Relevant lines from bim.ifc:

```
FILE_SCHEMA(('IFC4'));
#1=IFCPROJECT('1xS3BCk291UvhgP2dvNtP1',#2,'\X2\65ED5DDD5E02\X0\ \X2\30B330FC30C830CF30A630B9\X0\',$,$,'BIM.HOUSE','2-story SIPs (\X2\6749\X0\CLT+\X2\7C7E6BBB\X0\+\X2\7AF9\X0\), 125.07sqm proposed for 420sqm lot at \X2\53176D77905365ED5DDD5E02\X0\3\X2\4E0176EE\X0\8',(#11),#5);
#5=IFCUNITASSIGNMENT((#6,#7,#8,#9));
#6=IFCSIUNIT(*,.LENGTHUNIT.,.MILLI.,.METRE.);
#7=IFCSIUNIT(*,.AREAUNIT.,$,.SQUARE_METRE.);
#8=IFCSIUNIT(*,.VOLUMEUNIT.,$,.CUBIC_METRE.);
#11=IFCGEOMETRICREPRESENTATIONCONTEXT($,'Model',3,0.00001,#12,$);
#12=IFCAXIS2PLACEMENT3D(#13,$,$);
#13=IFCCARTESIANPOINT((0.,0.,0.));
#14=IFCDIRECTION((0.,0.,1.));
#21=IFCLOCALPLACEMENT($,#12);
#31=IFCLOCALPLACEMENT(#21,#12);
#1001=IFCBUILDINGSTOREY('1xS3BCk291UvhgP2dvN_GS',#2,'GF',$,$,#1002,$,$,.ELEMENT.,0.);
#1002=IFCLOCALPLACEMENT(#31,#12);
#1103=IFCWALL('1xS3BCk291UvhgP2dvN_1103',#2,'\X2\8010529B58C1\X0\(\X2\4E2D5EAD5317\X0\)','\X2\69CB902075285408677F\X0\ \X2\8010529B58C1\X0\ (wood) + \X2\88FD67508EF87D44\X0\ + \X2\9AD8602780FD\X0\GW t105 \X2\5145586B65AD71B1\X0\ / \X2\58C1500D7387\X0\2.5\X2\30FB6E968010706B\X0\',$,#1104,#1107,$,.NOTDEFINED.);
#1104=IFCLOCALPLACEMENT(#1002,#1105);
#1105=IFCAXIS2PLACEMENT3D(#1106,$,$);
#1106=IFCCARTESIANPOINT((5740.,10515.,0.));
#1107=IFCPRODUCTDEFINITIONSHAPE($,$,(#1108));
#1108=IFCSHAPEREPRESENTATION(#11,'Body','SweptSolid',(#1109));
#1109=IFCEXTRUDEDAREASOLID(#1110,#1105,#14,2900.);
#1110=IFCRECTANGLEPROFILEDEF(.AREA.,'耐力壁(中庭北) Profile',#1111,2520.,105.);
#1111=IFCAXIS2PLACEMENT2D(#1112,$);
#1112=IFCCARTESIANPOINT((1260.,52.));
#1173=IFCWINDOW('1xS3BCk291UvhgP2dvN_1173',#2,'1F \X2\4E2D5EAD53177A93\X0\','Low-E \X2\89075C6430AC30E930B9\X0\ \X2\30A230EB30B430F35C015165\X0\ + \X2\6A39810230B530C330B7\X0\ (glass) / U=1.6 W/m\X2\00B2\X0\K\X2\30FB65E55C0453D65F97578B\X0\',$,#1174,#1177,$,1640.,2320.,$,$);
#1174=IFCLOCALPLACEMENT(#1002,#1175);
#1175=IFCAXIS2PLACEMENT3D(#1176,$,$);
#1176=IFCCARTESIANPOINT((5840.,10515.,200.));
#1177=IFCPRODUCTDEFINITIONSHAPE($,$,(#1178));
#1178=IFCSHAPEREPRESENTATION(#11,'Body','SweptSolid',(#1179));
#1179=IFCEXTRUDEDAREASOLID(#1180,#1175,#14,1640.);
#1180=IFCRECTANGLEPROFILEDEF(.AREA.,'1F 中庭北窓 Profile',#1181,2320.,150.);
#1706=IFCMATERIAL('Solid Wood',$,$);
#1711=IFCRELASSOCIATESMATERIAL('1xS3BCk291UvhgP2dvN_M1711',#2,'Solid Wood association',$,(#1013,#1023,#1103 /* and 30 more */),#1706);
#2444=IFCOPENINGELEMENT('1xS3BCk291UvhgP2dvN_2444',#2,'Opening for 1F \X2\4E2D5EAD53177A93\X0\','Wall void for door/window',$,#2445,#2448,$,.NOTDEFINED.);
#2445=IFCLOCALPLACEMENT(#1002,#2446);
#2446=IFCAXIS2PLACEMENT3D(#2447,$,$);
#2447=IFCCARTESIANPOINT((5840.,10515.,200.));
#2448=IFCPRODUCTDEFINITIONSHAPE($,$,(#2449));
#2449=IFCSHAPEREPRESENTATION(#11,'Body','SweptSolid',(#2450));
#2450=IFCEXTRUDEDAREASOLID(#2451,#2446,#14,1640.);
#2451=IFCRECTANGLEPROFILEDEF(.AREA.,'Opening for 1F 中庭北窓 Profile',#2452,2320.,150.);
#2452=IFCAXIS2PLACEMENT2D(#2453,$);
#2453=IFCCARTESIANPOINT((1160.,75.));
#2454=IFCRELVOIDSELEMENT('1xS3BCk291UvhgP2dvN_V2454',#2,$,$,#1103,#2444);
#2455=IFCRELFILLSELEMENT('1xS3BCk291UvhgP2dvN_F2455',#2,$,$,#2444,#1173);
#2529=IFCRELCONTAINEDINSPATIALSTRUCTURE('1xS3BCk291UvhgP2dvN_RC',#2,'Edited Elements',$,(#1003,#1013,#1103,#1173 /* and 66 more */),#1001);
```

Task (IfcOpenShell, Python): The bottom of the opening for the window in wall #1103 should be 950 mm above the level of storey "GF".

```python
import numpy as np
import ifcopenshell
import ifcopenshell.api.geometry
import ifcopenshell.geom
import ifcopenshell.util.element
import ifcopenshell.util.placement
import ifcopenshell.util.shape
import ifcopenshell.util.unit

model = ifcopenshell.open("bim.ifc")
unit_scale = ifcopenshell.util.unit.calculate_unit_scale(model)

window = model.by_id(1173)
opening = window.FillsVoids[0].RelatingOpeningElement
storey = ifcopenshell.util.element.get_container(window, ifc_class="IfcBuildingStorey")
level = ifcopenshell.util.placement.get_local_placement(storey.ObjectPlacement)[2, 3]

# The opening's origin need not be at the sill, so measure its lowest point.
shape = ifcopenshell.geom.create_shape(ifcopenshell.geom.settings(), opening)
bottom = ifcopenshell.util.shape.get_shape_bottom_elevation(shape, shape.geometry) / unit_scale
dz = level + 0.95 / unit_scale - bottom

shift = np.array([0.0, 0.0, dz])
# The window is not placed relative to its opening, so move both.
for product in (opening, window):
    matrix = ifcopenshell.util.placement.get_local_placement(product.ObjectPlacement)
    matrix[:3, 3] += shift
    ifcopenshell.api.geometry.edit_object_placement(model, product=product, matrix=matrix, is_si=False)

print(f"moved by {dz * unit_scale:+.3f} m")

model.write("bim-out.ifc")
```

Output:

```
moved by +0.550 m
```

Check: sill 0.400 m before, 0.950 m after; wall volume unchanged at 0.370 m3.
